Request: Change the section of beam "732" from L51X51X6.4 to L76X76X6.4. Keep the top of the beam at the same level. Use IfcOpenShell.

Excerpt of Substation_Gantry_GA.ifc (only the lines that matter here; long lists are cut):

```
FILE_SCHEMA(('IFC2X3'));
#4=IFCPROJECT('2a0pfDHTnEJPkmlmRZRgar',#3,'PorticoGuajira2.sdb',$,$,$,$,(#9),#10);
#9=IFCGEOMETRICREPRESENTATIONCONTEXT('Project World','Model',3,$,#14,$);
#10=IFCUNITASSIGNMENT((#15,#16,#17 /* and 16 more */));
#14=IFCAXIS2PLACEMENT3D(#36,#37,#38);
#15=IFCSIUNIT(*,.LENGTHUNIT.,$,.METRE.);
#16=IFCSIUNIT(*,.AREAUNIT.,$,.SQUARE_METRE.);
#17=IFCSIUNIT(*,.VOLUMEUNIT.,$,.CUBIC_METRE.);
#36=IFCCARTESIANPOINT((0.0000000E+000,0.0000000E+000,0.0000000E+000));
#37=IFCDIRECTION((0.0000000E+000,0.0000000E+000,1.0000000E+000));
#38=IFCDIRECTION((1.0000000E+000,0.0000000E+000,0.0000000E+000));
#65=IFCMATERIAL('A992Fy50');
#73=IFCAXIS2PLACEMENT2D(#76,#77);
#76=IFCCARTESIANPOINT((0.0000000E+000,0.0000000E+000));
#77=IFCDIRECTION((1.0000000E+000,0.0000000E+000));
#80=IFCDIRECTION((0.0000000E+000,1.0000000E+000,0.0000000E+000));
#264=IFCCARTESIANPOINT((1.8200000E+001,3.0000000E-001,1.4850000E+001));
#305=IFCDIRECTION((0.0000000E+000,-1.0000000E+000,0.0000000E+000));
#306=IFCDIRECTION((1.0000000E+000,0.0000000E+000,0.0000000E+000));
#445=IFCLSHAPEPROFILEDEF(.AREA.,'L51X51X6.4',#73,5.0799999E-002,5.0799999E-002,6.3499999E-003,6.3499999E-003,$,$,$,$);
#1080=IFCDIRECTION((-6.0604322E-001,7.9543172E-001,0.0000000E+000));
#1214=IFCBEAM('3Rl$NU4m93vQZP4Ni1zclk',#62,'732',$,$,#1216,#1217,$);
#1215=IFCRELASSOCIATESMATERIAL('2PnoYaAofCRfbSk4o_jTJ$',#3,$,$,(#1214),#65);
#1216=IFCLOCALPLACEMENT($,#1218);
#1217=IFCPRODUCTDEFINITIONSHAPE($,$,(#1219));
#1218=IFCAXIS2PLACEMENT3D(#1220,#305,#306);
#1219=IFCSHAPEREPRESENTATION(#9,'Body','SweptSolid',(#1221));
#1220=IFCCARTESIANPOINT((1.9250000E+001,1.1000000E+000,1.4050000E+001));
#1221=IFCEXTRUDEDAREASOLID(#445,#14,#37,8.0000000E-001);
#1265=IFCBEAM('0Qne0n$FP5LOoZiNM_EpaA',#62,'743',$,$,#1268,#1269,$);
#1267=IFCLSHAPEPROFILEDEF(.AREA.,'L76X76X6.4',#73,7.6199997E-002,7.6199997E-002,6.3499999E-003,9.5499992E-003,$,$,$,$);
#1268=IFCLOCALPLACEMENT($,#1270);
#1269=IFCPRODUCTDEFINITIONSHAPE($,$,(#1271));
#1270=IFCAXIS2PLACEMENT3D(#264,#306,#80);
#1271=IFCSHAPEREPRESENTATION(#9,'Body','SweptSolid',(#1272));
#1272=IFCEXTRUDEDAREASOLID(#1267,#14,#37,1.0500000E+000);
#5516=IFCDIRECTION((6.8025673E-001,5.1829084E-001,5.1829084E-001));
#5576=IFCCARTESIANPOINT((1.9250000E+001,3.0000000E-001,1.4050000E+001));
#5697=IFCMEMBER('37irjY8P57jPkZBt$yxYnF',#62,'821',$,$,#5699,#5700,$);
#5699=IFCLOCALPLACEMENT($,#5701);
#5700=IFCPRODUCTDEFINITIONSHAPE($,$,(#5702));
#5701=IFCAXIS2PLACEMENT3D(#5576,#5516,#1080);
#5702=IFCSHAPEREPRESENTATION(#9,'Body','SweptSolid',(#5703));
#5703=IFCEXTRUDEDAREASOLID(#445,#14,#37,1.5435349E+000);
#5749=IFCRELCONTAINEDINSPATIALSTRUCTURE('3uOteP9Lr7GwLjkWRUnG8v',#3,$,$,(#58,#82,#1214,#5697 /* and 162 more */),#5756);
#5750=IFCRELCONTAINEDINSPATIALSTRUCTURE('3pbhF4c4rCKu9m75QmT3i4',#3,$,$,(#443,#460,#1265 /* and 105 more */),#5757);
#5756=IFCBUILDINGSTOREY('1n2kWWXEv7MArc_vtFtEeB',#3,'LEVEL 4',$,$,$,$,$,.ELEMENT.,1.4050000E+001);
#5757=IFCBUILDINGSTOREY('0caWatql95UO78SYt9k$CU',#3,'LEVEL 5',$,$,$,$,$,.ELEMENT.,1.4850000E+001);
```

```python
import ifcopenshell
import ifcopenshell.util.element

model = ifcopenshell.open("Substation_Gantry_GA.ifc")

member = model.by_guid("3Rl$NU4m93vQZP4Ni1zclk")
source = next(p for p in model.by_type("IfcLShapeProfileDef") if p.ProfileName == "L76X76X6.4")

body = next(r for r in member.Representation.Representations if r.RepresentationIdentifier == "Body")
solid = body.Items[0]
old_profile = solid.SweptArea

# Copy the section's sizes but keep this member's own profile position.
profile = ifcopenshell.util.element.copy(model, source)
# Profiles are centred, so shift by half the change in depth to hold the top.
shift = (old_profile.Depth - profile.Depth) / 2
x, y = old_profile.Position.Location.Coordinates
up = (0.0, 1.0)  # upwards, in the solid's own plane
location = model.createIfcCartesianPoint((x + up[0] * shift, y + up[1] * shift))
profile.Position = model.createIfcAxis2Placement2D(location, old_profile.Position.RefDirection)
solid.SweptArea = profile
if not model.get_total_inverses(old_profile):
    ifcopenshell.util.element.remove_deep2(model, old_profile)

print(solid.SweptArea)

model.write("Substation_Gantry_GA_rev.ifc")
```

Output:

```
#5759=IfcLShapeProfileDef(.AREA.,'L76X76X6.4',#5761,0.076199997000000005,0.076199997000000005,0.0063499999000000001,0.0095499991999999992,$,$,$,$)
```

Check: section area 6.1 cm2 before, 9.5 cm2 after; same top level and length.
